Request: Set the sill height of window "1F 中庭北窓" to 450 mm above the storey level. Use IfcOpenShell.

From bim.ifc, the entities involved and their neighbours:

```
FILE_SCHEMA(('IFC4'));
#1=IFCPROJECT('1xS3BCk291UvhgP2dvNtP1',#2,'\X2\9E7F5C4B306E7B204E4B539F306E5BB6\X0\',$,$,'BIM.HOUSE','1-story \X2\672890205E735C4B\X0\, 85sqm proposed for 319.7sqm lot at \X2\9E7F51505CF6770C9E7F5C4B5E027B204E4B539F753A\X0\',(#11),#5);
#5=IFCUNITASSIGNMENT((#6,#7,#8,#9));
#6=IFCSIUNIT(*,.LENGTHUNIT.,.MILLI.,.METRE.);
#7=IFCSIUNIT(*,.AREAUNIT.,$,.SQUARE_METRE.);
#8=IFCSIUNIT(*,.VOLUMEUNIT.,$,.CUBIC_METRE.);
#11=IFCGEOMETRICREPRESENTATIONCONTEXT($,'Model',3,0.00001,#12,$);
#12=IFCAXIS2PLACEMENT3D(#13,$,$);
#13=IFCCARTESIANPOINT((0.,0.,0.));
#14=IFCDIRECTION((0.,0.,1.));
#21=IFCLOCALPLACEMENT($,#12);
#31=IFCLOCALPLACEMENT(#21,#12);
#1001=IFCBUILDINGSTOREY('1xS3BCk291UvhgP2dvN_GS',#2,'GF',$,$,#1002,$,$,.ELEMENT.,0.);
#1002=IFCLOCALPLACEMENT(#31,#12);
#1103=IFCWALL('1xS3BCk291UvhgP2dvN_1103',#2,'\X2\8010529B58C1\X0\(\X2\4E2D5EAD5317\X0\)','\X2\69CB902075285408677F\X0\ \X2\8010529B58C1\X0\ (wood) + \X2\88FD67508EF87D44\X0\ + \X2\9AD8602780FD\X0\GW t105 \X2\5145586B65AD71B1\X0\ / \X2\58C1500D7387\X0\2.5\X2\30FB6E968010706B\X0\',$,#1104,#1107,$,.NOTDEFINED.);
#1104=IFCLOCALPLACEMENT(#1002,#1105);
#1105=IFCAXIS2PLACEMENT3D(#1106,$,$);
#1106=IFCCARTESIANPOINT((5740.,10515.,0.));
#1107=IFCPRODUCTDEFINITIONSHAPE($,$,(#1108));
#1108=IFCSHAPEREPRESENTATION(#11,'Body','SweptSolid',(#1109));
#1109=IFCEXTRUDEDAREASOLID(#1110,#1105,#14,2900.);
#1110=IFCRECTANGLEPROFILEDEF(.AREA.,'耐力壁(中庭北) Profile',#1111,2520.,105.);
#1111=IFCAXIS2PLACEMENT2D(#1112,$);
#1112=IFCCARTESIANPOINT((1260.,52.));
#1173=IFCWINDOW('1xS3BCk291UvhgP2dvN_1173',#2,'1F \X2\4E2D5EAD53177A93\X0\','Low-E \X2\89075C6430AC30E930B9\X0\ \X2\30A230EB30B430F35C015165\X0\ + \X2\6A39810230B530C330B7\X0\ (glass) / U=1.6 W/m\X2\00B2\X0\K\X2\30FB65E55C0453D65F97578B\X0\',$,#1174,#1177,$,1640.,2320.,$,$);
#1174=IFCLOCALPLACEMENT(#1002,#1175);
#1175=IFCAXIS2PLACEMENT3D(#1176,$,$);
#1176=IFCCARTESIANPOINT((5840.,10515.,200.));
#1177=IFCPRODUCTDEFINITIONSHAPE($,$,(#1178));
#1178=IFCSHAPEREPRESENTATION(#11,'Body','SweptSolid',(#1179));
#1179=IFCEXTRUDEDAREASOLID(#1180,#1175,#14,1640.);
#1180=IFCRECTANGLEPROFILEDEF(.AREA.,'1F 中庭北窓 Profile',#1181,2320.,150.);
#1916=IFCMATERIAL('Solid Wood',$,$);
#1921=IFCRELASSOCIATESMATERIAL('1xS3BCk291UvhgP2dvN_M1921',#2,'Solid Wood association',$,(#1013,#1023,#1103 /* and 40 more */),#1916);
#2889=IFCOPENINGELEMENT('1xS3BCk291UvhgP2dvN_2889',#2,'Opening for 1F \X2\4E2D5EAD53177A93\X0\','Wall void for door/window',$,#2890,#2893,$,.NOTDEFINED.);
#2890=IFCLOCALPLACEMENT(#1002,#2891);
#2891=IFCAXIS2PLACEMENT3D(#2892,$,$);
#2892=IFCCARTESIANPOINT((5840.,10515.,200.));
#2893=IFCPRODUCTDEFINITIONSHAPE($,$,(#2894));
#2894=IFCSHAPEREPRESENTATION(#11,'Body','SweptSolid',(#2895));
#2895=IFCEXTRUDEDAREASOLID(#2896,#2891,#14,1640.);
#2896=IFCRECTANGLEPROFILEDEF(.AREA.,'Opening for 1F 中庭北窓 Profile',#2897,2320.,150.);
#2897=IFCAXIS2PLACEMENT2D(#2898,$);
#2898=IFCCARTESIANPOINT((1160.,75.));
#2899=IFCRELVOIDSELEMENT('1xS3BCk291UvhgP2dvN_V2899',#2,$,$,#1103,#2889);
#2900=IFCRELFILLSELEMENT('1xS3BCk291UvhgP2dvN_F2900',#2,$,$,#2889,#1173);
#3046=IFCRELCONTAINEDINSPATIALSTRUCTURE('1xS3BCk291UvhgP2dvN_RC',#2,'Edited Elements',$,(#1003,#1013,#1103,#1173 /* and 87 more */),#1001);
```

```python
import numpy as np
import ifcopenshell
import ifcopenshell.api.geometry
import ifcopenshell.geom
import ifcopenshell.util.element
import ifcopenshell.util.placement
import ifcopenshell.util.shape
import ifcopenshell.util.unit

model = ifcopenshell.open("bim.ifc")
unit_scale = ifcopenshell.util.unit.calculate_unit_scale(model)

window = model.by_guid("1xS3BCk291UvhgP2dvN_1173")
opening = window.FillsVoids[0].RelatingOpeningElement
storey = ifcopenshell.util.element.get_container(window, ifc_class="IfcBuildingStorey")
level = ifcopenshell.util.placement.get_local_placement(storey.ObjectPlacement)[2, 3]

# The opening's origin need not be at the sill, so measure its lowest point.
shape = ifcopenshell.geom.create_shape(ifcopenshell.geom.settings(), opening)
bottom = ifcopenshell.util.shape.get_shape_bottom_elevation(shape, shape.geometry) / unit_scale
dz = level + 0.45 / unit_scale - bottom

shift = np.array([0.0, 0.0, dz])
# The window is not placed relative to its opening, so move both.
for product in (opening, window):
    matrix = ifcopenshell.util.placement.get_local_placement(product.ObjectPlacement)
    matrix[:3, 3] += shift
    ifcopenshell.api.geometry.edit_object_placement(model, product=product, matrix=matrix, is_si=False)

print(f"moved by {dz * unit_scale:+.3f} m")

model.write("bim_rev.ifc")
```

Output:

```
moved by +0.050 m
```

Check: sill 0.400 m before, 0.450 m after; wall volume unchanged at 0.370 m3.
